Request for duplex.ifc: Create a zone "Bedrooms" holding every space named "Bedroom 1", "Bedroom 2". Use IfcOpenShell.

First a look at what the model holds.

```python
import ifcopenshell

model = ifcopenshell.open("duplex.ifc")
print(model.schema)
seen = {}
for space in model.by_type("IfcSpace"):
    seen[space.LongName] = seen.get(space.LongName, 0) + 1
for name, count in sorted(seen.items(), key=str):
    print(count, "x", name)
print("zones:", [z.Name for z in model.by_type("IfcZone")][:20])
```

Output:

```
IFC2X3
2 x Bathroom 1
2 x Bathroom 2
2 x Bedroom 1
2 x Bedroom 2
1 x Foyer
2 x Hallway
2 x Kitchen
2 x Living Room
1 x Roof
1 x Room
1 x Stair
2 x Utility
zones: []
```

```python
import ifcopenshell
import ifcopenshell.api.group
import ifcopenshell.api.root

model = ifcopenshell.open("duplex.ifc")

names = {"Bedroom 1", "Bedroom 2"}
spaces = [s for s in model.by_type("IfcSpace") if s.LongName in names]

zone = ifcopenshell.api.root.create_entity(model, ifc_class="IfcZone", name="Bedrooms")
ifcopenshell.api.group.assign_group(model, products=spaces, group=zone)
print(len(spaces), "spaces in", zone.Name)

model.write("duplex-out.ifc")
```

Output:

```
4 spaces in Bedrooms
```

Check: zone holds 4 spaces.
